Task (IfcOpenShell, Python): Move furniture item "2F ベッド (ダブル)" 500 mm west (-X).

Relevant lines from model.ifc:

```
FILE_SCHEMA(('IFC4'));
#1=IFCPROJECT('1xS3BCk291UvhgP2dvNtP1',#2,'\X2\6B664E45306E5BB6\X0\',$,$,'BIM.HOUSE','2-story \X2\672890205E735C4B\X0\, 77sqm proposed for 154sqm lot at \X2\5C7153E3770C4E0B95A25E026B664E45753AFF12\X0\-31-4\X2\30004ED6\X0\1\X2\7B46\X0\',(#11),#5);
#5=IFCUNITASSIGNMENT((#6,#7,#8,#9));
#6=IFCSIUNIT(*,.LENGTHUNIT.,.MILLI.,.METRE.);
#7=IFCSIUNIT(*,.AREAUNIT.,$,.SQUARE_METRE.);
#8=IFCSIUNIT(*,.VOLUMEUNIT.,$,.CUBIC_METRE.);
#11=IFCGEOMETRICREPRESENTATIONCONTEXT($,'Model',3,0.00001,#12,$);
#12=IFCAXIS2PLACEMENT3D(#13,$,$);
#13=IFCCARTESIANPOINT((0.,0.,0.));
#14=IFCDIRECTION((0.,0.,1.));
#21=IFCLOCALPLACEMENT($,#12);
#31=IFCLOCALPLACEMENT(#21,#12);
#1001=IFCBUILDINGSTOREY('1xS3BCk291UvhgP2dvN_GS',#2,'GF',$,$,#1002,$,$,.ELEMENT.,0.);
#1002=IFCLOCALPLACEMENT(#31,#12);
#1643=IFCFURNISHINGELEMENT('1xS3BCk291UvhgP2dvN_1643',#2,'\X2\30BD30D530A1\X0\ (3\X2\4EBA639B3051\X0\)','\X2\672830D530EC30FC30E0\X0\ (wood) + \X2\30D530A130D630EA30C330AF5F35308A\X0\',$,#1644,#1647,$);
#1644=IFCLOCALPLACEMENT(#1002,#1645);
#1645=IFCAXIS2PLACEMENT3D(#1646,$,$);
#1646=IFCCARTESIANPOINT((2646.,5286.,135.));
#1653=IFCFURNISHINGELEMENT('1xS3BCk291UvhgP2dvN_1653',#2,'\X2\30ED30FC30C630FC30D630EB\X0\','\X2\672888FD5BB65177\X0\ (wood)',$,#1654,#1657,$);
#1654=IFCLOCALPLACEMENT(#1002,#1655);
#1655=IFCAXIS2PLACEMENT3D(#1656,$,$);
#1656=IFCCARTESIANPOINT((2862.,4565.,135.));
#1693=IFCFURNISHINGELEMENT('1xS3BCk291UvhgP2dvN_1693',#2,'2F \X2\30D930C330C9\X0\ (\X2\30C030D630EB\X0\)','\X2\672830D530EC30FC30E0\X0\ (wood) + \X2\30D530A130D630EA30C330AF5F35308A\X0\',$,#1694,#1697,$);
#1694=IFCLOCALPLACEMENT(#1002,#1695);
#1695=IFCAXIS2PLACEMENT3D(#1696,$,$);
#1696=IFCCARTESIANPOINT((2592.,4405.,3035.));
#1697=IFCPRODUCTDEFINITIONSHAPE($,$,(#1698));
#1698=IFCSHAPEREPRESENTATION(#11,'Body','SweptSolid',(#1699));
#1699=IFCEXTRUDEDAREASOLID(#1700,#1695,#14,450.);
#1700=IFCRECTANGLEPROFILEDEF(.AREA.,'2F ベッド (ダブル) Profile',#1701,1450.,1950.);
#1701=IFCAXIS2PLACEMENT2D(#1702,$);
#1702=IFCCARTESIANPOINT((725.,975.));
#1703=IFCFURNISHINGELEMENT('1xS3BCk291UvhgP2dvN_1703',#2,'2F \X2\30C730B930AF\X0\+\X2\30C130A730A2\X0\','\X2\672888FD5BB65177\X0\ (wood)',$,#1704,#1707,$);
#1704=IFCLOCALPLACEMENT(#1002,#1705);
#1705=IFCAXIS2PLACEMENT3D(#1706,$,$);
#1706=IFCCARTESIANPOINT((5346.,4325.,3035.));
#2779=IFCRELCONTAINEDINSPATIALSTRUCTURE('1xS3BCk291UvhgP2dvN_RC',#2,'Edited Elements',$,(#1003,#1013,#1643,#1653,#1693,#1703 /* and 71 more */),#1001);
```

```python
import ifcopenshell
import ifcopenshell.api.geometry
import ifcopenshell.util.placement
import ifcopenshell.util.unit

model = ifcopenshell.open("model.ifc")
unit_scale = ifcopenshell.util.unit.calculate_unit_scale(model)

item = model.by_guid("1xS3BCk291UvhgP2dvN_1693")
matrix = ifcopenshell.util.placement.get_local_placement(item.ObjectPlacement)
matrix[0, 3] -= 0.5 / unit_scale
ifcopenshell.api.geometry.edit_object_placement(model, product=item, matrix=matrix, is_si=False)

print(ifcopenshell.util.placement.get_local_placement(item.ObjectPlacement).round(3) + 0.0)

model.write("model_updated.ifc")
```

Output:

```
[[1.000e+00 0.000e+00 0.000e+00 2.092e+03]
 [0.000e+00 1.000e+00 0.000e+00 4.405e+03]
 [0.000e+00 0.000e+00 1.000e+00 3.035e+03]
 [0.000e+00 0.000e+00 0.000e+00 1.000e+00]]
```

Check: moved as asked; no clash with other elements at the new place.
